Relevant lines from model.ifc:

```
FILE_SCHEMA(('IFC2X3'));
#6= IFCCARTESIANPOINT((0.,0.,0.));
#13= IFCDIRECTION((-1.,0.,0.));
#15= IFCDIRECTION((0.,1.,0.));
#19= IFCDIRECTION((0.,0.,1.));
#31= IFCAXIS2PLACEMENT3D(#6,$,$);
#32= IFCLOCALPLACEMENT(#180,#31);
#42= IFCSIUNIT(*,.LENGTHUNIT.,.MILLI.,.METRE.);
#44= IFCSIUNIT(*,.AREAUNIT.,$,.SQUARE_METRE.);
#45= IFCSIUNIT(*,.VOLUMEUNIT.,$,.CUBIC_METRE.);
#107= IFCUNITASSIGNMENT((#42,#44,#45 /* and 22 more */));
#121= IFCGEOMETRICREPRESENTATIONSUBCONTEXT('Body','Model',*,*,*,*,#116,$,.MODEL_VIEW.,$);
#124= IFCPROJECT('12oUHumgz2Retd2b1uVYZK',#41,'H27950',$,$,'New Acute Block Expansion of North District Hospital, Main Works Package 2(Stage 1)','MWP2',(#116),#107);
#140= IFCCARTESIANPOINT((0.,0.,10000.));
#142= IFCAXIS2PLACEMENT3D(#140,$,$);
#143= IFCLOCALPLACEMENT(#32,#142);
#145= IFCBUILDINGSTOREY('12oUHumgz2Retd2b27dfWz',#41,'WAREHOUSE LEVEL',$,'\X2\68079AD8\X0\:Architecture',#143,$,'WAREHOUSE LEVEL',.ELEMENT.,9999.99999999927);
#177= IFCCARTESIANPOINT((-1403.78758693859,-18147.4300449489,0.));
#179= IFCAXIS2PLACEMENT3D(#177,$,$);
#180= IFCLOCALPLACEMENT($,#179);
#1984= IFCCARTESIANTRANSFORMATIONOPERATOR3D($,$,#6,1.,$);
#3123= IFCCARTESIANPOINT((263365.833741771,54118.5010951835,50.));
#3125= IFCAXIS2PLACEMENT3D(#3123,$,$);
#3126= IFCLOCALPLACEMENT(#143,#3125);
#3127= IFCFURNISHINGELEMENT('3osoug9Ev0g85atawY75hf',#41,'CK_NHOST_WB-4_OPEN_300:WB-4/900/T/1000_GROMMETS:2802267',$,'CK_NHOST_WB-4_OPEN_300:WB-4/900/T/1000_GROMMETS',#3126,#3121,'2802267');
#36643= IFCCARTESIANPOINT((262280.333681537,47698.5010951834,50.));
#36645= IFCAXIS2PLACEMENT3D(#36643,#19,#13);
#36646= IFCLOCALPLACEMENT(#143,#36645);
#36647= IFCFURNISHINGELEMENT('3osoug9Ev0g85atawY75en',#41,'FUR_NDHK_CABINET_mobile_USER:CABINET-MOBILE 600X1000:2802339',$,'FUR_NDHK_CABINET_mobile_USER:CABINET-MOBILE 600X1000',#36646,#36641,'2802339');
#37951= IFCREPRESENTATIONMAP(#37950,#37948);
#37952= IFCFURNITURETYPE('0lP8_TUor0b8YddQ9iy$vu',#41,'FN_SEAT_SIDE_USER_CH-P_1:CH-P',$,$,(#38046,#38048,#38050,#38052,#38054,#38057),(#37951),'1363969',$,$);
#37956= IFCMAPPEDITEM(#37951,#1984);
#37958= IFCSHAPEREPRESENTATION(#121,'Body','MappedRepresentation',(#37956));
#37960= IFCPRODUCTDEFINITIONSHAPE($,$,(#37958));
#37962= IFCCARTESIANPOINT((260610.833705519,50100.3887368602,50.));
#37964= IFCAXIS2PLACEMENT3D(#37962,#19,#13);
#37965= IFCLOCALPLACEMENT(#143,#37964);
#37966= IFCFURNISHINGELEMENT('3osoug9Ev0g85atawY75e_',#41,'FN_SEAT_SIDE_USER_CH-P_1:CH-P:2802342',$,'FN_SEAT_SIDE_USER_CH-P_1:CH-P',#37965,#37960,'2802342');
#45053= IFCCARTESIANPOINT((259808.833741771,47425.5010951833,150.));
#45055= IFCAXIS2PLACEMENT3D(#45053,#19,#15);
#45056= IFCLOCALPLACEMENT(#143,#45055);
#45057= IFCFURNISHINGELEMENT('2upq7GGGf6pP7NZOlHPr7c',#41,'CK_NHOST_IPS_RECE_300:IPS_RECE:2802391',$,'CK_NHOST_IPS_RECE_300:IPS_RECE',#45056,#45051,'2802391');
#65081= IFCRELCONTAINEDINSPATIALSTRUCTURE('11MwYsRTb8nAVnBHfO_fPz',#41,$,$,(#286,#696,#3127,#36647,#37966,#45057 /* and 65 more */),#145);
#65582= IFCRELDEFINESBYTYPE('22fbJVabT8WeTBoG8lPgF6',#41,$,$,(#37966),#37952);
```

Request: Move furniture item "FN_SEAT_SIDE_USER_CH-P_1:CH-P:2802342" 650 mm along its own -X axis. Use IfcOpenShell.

```python
import ifcopenshell
import ifcopenshell.api.geometry
import ifcopenshell.util.placement
import ifcopenshell.util.unit

model = ifcopenshell.open("model.ifc")
unit_scale = ifcopenshell.util.unit.calculate_unit_scale(model)

item = model.by_guid("3osoug9Ev0g85atawY75e_")
matrix = ifcopenshell.util.placement.get_local_placement(item.ObjectPlacement)
matrix[:3, 3] -= matrix[:3, 0] * 0.65 / unit_scale
ifcopenshell.api.geometry.edit_object_placement(model, product=item, matrix=matrix, is_si=False)

print(ifcopenshell.util.placement.get_local_placement(item.ObjectPlacement).round(3) + 0.0)

model.write("model_updated.ifc")
```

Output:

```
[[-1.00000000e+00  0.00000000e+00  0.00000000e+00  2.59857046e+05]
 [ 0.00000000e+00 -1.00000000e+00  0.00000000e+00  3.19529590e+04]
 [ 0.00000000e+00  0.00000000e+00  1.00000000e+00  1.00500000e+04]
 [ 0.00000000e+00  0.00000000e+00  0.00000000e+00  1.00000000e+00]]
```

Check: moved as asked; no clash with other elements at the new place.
